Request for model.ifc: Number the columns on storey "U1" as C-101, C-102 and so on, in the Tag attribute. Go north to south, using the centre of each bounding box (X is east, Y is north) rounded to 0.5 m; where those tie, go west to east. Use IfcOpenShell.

First a look at what the model holds.

```python
import ifcopenshell
import ifcopenshell.util.element
import ifcopenshell.util.placement

model = ifcopenshell.open("model.ifc")
print(model.schema)
storey = next(s for s in model.by_type("IfcBuildingStorey") if s.Name == "U1")
columns = [e for e in ifcopenshell.util.element.get_decomposition(storey) if e.is_a("IfcColumn")]
for e in sorted(columns, key=lambda e: e.id()):
    origin = ifcopenshell.util.placement.get_local_placement(e.ObjectPlacement)[:3, 3]
    print(e.id(), e.Tag, e.Name, origin.round(2) + 0.0, sep=" | ")
```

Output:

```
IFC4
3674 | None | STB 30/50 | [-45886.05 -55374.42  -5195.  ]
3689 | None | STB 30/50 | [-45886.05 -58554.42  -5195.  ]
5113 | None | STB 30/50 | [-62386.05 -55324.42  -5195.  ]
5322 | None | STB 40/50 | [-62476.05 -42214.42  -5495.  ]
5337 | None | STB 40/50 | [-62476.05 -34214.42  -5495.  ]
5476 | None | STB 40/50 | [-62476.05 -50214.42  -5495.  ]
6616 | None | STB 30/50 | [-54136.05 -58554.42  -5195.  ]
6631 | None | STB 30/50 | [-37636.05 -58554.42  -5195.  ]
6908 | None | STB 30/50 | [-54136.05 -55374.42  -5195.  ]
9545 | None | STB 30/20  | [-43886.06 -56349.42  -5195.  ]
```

```python
import ifcopenshell
import ifcopenshell.geom
import ifcopenshell.util.element
import ifcopenshell.util.shape

model = ifcopenshell.open("model.ifc")
settings = ifcopenshell.geom.settings()
settings.set("use-world-coords", True)


def centre(element):
    shape = ifcopenshell.geom.create_shape(settings, element)
    return ifcopenshell.util.shape.get_bbox_centroid(shape.geometry)


storey = next(s for s in model.by_type("IfcBuildingStorey") if s.Name == "U1")
columns = [e for e in ifcopenshell.util.element.get_decomposition(storey) if e.is_a("IfcColumn")]

# Insertion points can sit at a corner or the storey origin, so sort by the geometry (in metres).
centres = {e: centre(e) for e in columns}
columns.sort(key=lambda e: (-round(centres[e][1] / 0.5), centres[e][0]))

for i, e in enumerate(columns, start=1):
    number = f"C-1{i:02d}"
    e.Tag = number
    print(e.id(), number)

model.write("model_updated.ifc")
```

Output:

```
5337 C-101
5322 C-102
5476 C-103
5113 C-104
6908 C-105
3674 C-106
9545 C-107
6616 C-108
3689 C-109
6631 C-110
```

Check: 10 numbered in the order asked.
